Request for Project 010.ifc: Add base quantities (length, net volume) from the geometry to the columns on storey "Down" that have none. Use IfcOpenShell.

First a look at what the model holds.

```python
import ifcopenshell
import ifcopenshell.util.element
import ifcopenshell.util.unit

model = ifcopenshell.open("Project 010.ifc")
print(model.schema)
for unit_type in ("LENGTHUNIT", "AREAUNIT", "VOLUMEUNIT"):
    print(unit_type, ifcopenshell.util.unit.calculate_unit_scale(model, unit_type))
storey = next(s for s in model.by_type("IfcBuildingStorey") if s.Name == "Down")
columns = [e for e in ifcopenshell.util.element.get_decomposition(storey) if e.is_a("IfcColumn")]
for e in sorted(columns, key=lambda e: e.id()):
    print(e.id(), e.is_a(), e.Name, list(ifcopenshell.util.element.get_psets(e, qtos_only=True)), sep=" | ")
```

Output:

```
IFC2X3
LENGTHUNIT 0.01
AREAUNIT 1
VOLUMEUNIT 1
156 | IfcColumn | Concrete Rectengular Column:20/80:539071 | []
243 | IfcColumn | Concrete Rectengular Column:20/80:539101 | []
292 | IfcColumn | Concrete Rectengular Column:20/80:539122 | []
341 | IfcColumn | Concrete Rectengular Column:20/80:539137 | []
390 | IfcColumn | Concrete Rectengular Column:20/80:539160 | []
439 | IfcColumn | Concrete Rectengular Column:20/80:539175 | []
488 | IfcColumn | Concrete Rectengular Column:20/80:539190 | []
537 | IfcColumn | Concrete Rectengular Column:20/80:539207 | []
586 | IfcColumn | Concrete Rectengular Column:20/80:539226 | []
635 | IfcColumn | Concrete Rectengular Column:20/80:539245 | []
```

```python
import ifcopenshell
import ifcopenshell.api.pset
import ifcopenshell.geom
import ifcopenshell.util.element
import ifcopenshell.util.shape
import ifcopenshell.util.unit

model = ifcopenshell.open("Project 010.ifc")
unit_scale = ifcopenshell.util.unit.calculate_unit_scale(model)
volume_scale = ifcopenshell.util.unit.calculate_unit_scale(model, "VOLUMEUNIT")
settings = ifcopenshell.geom.settings()

storey = next(s for s in model.by_type("IfcBuildingStorey") if s.Name == "Down")
columns = [e for e in ifcopenshell.util.element.get_decomposition(storey) if e.is_a("IfcColumn")]

for e in sorted(columns, key=lambda e: e.id()):
    if ifcopenshell.util.element.get_psets(e, qtos_only=True, should_inherit=False):
        continue
    # Geometry comes back in metres, in the element's own axes.
    shape = ifcopenshell.geom.create_shape(settings, e)
    values = {
        "Length": ifcopenshell.util.shape.get_z(shape.geometry) / unit_scale,
        "NetVolume": ifcopenshell.util.shape.get_volume(shape.geometry) / volume_scale,
    }
    qto = ifcopenshell.api.pset.add_qto(model, product=e, name="BaseQuantities")
    ifcopenshell.api.pset.edit_qto(model, qto=qto, properties=values)
    print(e.id(), {k: round(v, 3) for k, v in values.items()})

model.write("Project 010_rev.ifc")
```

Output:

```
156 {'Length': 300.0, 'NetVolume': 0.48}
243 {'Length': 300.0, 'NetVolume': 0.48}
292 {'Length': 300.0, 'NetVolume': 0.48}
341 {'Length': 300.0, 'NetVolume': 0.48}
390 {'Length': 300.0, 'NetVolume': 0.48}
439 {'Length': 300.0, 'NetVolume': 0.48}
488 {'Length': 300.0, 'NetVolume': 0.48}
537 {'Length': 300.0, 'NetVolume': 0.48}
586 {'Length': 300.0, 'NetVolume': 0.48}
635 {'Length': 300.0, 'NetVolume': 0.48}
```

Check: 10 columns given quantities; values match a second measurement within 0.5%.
